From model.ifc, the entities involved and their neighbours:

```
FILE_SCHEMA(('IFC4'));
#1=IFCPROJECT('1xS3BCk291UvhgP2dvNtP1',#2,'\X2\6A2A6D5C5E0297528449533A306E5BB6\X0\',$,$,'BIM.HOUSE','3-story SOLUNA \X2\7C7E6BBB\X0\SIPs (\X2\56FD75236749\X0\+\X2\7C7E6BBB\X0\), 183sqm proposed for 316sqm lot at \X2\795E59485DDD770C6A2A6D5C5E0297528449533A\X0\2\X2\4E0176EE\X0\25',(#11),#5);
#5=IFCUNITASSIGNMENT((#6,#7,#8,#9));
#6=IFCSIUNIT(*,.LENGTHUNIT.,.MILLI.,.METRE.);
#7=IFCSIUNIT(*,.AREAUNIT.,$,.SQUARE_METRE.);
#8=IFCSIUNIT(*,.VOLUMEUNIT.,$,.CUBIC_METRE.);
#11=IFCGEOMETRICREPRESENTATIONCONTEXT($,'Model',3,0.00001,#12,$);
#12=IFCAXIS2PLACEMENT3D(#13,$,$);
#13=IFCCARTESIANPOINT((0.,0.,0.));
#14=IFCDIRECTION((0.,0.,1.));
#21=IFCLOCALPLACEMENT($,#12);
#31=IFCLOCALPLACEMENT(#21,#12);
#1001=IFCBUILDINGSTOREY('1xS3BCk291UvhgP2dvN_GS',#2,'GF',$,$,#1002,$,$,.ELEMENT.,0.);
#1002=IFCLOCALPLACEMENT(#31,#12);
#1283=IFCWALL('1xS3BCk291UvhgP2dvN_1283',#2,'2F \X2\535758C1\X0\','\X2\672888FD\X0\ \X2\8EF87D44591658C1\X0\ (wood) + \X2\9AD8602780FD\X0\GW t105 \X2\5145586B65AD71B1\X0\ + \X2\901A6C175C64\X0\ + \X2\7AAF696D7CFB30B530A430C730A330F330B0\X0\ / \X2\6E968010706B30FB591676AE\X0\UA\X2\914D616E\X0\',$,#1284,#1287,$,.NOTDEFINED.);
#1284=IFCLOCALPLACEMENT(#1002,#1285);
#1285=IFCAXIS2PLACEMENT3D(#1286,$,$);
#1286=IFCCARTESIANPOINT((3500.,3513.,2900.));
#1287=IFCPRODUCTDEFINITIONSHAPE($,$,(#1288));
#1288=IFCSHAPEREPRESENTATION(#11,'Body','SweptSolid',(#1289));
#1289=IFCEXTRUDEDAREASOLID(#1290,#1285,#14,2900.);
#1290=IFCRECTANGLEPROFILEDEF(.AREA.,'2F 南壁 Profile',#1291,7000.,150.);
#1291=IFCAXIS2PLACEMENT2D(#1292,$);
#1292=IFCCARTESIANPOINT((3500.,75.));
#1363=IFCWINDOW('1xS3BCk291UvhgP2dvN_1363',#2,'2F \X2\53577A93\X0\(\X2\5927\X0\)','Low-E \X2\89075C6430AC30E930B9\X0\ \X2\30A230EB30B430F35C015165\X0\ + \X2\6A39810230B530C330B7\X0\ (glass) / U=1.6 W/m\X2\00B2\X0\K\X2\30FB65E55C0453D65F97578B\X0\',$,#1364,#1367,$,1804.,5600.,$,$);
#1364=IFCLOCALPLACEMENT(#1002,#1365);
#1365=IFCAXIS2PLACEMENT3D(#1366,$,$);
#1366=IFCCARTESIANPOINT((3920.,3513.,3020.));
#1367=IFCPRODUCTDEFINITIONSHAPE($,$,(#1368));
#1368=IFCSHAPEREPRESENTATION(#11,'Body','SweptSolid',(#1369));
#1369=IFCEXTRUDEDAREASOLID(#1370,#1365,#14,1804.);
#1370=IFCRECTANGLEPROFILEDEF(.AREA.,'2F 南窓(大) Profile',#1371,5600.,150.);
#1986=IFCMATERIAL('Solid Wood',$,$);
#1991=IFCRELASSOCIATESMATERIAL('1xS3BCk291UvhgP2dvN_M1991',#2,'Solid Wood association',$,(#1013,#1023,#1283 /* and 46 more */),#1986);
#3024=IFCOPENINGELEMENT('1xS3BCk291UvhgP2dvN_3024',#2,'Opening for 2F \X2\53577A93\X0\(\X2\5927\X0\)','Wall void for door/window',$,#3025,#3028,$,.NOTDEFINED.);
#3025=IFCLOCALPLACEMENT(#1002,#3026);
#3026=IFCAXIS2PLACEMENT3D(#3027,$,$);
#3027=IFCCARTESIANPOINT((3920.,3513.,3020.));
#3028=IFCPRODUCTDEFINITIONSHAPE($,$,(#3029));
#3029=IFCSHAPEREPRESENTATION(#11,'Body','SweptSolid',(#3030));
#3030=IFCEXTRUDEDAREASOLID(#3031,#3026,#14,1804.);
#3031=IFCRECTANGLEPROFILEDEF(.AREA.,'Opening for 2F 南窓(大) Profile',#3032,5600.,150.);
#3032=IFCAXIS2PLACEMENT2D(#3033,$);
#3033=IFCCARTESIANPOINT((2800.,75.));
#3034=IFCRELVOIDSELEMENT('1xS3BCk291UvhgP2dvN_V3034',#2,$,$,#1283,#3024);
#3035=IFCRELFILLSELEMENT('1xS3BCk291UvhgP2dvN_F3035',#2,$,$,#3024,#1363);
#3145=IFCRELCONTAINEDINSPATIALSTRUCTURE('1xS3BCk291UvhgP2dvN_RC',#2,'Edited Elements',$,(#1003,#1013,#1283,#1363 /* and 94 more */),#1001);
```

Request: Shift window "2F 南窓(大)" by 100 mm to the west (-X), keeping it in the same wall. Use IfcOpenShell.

```python
import ifcopenshell
import ifcopenshell.api.geometry
import ifcopenshell.util.placement
import ifcopenshell.util.unit

model = ifcopenshell.open("model.ifc")
unit_scale = ifcopenshell.util.unit.calculate_unit_scale(model)

window = model.by_guid("1xS3BCk291UvhgP2dvN_1363")
opening = window.FillsVoids[0].RelatingOpeningElement
wall = opening.VoidsElements[0].RelatingBuildingElement

wall_matrix = ifcopenshell.util.placement.get_local_placement(wall.ObjectPlacement)
shift = wall_matrix[:3, 0] * -0.1 / unit_scale
before = ifcopenshell.util.placement.get_local_placement(window.ObjectPlacement)[:3, 3].copy()

# The window is not placed relative to its opening, so move both.
for product in (opening, window):
    matrix = ifcopenshell.util.placement.get_local_placement(product.ObjectPlacement)
    matrix[:3, 3] += shift
    ifcopenshell.api.geometry.edit_object_placement(model, product=product, matrix=matrix, is_si=False)

after = ifcopenshell.util.placement.get_local_placement(window.ObjectPlacement)[:3, 3]
print("window moved by", (after - before).round(3) + 0.0)

model.write("model_v2.ifc")
```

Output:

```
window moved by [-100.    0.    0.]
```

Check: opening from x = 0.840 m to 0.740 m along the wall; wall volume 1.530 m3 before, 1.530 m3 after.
